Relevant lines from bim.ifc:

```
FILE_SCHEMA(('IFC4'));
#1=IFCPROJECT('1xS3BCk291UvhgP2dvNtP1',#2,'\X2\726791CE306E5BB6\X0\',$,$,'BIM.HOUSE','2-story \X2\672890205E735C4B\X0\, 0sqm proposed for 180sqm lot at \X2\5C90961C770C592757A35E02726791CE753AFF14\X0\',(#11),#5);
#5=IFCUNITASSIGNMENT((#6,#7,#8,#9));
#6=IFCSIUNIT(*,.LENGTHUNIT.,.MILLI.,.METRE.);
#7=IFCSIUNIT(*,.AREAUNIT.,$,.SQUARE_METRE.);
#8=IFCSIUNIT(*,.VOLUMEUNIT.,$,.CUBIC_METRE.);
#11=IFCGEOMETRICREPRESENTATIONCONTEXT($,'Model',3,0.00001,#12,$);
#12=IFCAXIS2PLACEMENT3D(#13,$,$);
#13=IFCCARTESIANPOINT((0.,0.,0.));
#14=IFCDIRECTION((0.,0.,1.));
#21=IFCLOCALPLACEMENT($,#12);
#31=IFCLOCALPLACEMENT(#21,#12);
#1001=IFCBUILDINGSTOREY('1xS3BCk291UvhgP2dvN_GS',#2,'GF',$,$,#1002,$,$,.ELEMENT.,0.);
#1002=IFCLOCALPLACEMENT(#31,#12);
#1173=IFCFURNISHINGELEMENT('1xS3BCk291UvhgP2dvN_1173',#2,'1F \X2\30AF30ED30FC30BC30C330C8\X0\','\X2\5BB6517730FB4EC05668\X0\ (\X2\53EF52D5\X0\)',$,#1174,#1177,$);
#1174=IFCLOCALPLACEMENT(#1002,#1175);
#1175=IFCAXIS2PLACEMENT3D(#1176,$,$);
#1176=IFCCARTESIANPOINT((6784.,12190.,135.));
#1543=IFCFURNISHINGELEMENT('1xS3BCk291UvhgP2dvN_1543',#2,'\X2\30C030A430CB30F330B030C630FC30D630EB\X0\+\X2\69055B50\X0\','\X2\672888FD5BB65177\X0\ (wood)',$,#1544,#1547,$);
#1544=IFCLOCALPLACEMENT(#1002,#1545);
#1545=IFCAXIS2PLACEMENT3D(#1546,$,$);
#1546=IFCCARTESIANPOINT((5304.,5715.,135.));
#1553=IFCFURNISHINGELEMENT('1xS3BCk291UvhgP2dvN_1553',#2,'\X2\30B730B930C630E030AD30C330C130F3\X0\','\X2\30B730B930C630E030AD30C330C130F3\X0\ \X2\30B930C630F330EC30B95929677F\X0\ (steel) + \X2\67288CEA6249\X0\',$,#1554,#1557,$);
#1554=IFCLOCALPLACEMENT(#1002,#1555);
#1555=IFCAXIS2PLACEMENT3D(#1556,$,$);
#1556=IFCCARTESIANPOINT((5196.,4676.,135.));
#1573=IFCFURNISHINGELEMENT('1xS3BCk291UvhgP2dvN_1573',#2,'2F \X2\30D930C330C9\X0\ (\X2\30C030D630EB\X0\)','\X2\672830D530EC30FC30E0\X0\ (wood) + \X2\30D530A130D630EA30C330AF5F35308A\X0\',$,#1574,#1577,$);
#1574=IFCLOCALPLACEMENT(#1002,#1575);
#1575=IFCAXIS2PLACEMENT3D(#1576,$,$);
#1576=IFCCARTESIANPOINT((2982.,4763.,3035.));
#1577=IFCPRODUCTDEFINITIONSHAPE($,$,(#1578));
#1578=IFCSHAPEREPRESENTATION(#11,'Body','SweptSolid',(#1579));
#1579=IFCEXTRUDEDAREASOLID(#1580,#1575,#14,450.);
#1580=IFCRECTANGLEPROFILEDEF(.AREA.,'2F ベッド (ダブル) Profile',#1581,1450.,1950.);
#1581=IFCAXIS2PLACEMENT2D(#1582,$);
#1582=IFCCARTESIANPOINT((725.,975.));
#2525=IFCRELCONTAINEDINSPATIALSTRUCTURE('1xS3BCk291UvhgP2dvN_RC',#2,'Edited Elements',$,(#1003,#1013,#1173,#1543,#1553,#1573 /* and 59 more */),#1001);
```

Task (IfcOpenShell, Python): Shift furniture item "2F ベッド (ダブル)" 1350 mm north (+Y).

```python
import ifcopenshell
import ifcopenshell.api.geometry
import ifcopenshell.util.placement

model = ifcopenshell.open("bim.ifc")

item = model.by_guid("1xS3BCk291UvhgP2dvN_1573")
matrix = ifcopenshell.util.placement.get_local_placement(item.ObjectPlacement)
matrix[1, 3] += 1350.0
ifcopenshell.api.geometry.edit_object_placement(model, product=item, matrix=matrix, is_si=False)

print(ifcopenshell.util.placement.get_local_placement(item.ObjectPlacement).round(3) + 0.0)

model.write("bim_rev.ifc")
```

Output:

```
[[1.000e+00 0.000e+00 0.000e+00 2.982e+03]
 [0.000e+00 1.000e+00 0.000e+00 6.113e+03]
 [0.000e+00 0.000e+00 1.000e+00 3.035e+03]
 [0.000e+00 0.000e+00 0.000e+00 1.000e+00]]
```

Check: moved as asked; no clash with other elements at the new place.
